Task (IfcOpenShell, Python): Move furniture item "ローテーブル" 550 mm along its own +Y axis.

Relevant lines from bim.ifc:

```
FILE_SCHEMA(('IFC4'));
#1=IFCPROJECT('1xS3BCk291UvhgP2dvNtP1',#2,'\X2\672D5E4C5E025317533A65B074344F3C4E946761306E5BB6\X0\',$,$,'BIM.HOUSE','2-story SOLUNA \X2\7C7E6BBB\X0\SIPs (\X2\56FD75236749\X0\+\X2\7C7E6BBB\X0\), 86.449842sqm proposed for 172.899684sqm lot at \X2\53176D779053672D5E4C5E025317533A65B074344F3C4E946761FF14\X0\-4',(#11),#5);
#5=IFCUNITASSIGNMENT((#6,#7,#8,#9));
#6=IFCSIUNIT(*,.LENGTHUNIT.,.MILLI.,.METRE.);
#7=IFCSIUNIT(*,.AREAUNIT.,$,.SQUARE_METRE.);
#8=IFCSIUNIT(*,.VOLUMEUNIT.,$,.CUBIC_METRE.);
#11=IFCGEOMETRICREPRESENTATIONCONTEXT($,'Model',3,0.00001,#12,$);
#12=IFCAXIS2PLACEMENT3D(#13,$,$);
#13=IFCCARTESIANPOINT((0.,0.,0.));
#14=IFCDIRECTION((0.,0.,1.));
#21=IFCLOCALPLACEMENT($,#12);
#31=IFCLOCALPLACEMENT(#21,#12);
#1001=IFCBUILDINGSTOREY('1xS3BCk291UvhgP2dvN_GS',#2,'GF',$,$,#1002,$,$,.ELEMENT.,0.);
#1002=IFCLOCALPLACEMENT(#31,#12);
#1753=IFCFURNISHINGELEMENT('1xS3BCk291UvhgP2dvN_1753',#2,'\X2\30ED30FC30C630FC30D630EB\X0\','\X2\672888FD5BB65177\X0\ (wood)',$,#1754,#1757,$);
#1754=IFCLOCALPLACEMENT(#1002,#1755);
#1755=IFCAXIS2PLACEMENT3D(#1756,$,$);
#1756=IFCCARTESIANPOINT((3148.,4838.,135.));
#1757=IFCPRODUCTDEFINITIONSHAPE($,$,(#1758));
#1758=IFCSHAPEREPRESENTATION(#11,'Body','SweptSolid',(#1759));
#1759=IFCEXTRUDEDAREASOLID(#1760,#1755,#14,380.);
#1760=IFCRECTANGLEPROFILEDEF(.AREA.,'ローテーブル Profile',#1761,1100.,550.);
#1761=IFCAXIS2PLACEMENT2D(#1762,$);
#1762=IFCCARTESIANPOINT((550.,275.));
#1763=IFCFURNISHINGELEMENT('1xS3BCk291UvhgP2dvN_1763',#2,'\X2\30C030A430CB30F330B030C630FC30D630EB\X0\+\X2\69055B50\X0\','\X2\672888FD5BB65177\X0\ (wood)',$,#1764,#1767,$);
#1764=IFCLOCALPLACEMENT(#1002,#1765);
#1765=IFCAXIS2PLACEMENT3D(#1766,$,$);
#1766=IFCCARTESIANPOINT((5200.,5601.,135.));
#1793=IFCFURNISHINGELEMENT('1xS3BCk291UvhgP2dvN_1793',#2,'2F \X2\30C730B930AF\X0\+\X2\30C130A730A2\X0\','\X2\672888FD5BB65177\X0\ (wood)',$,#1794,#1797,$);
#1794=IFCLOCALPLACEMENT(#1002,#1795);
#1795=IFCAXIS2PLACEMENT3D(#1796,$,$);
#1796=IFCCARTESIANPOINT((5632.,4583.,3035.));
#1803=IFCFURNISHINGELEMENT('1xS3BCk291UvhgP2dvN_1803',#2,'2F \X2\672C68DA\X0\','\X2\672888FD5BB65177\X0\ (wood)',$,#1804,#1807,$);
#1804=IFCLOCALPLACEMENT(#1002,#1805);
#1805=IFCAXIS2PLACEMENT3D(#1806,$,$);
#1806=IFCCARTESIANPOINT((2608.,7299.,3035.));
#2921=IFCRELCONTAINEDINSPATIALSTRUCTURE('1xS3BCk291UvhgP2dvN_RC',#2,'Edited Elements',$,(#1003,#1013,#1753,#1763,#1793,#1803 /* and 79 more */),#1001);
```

```python
import ifcopenshell
import ifcopenshell.api.geometry
import ifcopenshell.util.placement

model = ifcopenshell.open("bim.ifc")

item = model.by_guid("1xS3BCk291UvhgP2dvN_1753")
matrix = ifcopenshell.util.placement.get_local_placement(item.ObjectPlacement)
matrix[:3, 3] += matrix[:3, 1] * 550.0
ifcopenshell.api.geometry.edit_object_placement(model, product=item, matrix=matrix, is_si=False)

print(ifcopenshell.util.placement.get_local_placement(item.ObjectPlacement).round(3) + 0.0)

model.write("bim_v2.ifc")
```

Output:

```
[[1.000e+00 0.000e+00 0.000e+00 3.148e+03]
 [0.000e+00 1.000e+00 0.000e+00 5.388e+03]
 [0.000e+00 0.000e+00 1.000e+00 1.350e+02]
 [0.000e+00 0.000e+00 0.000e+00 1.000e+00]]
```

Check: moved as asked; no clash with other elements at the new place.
